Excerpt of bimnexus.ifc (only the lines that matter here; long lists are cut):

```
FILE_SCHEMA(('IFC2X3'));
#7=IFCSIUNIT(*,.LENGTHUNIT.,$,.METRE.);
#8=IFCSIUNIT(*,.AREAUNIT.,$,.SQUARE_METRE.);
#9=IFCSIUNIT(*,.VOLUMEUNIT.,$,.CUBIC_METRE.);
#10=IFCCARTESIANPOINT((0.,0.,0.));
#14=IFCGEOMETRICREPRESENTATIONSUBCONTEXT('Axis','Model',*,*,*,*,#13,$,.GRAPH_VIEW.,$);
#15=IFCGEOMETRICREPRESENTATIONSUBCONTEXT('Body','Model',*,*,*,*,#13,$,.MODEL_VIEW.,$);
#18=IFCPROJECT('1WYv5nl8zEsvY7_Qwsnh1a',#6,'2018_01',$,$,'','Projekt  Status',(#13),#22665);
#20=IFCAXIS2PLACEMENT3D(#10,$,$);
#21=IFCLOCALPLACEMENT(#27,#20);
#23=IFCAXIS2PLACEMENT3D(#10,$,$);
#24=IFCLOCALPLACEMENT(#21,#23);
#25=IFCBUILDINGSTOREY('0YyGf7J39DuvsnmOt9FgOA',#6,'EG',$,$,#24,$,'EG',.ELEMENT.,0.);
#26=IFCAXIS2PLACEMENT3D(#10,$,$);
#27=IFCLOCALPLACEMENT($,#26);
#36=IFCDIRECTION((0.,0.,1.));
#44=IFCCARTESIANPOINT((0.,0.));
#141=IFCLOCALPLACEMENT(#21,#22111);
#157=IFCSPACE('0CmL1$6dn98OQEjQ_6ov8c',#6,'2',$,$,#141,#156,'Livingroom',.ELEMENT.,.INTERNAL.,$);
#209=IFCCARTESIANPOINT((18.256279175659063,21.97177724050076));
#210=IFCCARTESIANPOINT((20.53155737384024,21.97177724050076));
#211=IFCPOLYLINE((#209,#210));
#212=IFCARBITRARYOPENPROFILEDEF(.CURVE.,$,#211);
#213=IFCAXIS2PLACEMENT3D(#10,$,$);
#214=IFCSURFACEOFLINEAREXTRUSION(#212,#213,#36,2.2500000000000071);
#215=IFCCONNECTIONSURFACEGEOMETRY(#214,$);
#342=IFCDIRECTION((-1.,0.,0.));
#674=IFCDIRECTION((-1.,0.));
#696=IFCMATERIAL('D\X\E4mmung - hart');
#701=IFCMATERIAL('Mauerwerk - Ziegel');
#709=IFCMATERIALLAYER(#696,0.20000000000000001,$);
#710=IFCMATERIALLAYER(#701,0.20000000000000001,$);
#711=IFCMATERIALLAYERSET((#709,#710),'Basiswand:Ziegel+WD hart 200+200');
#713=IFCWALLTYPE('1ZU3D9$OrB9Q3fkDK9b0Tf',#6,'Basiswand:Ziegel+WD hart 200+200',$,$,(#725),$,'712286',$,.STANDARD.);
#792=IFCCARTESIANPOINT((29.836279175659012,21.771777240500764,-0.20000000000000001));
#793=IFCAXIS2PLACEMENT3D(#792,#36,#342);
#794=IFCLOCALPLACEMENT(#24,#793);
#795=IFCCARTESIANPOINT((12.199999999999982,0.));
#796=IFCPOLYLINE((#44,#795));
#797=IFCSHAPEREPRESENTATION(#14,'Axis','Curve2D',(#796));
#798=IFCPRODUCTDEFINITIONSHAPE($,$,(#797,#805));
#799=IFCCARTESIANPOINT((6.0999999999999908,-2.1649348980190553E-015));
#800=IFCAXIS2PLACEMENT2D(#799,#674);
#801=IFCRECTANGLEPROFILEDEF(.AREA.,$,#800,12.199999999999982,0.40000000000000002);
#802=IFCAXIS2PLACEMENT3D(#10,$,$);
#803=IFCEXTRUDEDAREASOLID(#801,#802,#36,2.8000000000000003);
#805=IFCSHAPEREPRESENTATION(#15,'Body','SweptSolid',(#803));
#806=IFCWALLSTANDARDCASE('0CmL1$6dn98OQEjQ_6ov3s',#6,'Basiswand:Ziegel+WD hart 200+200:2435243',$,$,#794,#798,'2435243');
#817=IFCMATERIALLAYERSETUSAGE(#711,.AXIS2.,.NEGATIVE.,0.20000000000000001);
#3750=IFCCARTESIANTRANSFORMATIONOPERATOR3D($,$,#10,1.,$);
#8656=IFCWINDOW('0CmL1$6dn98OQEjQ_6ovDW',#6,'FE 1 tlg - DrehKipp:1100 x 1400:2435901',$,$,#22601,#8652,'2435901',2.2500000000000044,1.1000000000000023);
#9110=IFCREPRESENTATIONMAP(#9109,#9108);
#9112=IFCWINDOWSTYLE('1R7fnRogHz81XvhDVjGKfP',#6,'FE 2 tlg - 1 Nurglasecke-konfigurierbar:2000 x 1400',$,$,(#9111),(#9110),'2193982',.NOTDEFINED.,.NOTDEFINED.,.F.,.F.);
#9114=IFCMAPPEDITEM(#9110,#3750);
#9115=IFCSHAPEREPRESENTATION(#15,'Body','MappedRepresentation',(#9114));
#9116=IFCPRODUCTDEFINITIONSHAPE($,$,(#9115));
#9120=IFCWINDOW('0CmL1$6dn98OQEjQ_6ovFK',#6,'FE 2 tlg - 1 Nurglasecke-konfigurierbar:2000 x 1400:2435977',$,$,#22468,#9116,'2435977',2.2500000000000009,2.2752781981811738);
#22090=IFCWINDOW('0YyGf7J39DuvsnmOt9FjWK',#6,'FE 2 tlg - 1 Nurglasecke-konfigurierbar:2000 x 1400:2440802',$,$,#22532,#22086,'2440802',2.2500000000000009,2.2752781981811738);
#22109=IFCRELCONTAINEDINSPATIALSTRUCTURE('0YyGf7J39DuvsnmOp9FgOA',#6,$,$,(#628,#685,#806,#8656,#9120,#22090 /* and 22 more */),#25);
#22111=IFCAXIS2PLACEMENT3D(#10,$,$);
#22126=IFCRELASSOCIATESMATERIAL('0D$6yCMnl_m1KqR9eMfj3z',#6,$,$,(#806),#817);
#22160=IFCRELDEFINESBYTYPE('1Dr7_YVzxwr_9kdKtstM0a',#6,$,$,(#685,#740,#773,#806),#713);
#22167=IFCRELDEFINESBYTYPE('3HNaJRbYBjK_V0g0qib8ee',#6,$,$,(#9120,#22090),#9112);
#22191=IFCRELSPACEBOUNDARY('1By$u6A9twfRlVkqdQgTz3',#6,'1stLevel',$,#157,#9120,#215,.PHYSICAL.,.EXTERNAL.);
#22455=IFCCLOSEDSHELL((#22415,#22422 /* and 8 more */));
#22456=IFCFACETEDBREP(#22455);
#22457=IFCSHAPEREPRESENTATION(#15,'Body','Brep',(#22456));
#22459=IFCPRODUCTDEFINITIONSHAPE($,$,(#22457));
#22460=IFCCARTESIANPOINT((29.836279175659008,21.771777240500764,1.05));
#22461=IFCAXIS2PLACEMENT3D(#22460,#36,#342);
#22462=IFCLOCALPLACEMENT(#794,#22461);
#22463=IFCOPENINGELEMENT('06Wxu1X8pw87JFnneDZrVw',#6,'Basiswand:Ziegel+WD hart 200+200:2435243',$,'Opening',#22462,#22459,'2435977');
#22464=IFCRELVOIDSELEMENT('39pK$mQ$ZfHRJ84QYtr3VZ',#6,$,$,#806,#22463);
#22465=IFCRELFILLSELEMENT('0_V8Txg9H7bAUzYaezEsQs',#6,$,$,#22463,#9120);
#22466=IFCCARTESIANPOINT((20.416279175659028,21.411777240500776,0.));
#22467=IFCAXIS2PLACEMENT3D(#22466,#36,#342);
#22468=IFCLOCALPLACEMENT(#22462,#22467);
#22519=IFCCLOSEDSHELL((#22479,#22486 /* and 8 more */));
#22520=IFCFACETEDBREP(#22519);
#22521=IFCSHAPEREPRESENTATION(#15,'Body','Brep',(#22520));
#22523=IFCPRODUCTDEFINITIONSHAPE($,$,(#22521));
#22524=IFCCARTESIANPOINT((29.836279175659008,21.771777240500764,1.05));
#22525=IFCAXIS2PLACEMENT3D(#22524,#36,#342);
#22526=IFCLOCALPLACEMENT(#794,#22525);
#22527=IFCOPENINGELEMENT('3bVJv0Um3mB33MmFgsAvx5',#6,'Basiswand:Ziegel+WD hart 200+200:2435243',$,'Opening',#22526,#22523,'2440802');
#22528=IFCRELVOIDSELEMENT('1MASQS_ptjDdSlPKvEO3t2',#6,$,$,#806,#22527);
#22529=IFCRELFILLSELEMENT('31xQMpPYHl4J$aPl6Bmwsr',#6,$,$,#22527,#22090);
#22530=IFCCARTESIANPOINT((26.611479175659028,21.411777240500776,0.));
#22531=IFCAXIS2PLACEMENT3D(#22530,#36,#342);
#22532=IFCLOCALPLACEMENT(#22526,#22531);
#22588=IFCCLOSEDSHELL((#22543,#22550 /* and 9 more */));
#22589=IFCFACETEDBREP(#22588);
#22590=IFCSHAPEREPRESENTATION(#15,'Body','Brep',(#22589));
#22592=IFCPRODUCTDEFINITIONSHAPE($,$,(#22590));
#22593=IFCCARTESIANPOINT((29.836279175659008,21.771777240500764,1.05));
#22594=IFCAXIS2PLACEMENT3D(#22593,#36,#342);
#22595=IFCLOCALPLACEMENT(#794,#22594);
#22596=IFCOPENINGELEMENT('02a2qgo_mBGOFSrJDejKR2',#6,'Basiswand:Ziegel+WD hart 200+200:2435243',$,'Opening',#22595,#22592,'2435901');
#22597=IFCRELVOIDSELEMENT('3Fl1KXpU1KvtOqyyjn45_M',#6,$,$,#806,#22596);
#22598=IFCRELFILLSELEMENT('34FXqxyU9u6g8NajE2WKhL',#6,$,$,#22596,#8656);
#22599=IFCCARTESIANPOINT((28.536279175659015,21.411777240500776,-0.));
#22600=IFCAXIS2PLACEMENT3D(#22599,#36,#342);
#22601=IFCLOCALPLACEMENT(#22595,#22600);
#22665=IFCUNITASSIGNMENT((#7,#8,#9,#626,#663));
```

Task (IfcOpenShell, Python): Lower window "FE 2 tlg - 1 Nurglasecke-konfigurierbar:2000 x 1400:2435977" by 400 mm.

```python
import numpy as np
import ifcopenshell
import ifcopenshell.api.geometry
import ifcopenshell.util.placement
import ifcopenshell.util.unit

model = ifcopenshell.open("bimnexus.ifc")
unit_scale = ifcopenshell.util.unit.calculate_unit_scale(model)

window = model.by_guid("0CmL1$6dn98OQEjQ_6ovFK")
opening = window.FillsVoids[0].RelatingOpeningElement
dz = -0.4 / unit_scale

shift = np.array([0.0, 0.0, dz])
# The window is placed relative to its opening, so it follows when the opening moves.
matrix = ifcopenshell.util.placement.get_local_placement(opening.ObjectPlacement)
matrix[:3, 3] += shift
ifcopenshell.api.geometry.edit_object_placement(
    model, product=opening, matrix=matrix, is_si=False, should_transform_children=True
)

# Space boundary surfaces are stored in each space's coordinates; move them too.
for rel in window.ProvidesBoundaries:
    if not rel.ConnectionGeometry:
        continue
    surface = rel.ConnectionGeometry.SurfaceOnRelatingElement
    space_matrix = ifcopenshell.util.placement.get_local_placement(rel.RelatingSpace.ObjectPlacement)
    point = np.array(surface.Position.Location.Coordinates) + space_matrix[:3, :3].T @ shift
    surface.Position = model.createIfcAxis2Placement3D(
        model.createIfcCartesianPoint(point.tolist()), surface.Position.Axis, surface.Position.RefDirection
    )

print(f"moved by {dz * unit_scale:+.3f} m")

model.write("bimnexus_rev.ifc")
```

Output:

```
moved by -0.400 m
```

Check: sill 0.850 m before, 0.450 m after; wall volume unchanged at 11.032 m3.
